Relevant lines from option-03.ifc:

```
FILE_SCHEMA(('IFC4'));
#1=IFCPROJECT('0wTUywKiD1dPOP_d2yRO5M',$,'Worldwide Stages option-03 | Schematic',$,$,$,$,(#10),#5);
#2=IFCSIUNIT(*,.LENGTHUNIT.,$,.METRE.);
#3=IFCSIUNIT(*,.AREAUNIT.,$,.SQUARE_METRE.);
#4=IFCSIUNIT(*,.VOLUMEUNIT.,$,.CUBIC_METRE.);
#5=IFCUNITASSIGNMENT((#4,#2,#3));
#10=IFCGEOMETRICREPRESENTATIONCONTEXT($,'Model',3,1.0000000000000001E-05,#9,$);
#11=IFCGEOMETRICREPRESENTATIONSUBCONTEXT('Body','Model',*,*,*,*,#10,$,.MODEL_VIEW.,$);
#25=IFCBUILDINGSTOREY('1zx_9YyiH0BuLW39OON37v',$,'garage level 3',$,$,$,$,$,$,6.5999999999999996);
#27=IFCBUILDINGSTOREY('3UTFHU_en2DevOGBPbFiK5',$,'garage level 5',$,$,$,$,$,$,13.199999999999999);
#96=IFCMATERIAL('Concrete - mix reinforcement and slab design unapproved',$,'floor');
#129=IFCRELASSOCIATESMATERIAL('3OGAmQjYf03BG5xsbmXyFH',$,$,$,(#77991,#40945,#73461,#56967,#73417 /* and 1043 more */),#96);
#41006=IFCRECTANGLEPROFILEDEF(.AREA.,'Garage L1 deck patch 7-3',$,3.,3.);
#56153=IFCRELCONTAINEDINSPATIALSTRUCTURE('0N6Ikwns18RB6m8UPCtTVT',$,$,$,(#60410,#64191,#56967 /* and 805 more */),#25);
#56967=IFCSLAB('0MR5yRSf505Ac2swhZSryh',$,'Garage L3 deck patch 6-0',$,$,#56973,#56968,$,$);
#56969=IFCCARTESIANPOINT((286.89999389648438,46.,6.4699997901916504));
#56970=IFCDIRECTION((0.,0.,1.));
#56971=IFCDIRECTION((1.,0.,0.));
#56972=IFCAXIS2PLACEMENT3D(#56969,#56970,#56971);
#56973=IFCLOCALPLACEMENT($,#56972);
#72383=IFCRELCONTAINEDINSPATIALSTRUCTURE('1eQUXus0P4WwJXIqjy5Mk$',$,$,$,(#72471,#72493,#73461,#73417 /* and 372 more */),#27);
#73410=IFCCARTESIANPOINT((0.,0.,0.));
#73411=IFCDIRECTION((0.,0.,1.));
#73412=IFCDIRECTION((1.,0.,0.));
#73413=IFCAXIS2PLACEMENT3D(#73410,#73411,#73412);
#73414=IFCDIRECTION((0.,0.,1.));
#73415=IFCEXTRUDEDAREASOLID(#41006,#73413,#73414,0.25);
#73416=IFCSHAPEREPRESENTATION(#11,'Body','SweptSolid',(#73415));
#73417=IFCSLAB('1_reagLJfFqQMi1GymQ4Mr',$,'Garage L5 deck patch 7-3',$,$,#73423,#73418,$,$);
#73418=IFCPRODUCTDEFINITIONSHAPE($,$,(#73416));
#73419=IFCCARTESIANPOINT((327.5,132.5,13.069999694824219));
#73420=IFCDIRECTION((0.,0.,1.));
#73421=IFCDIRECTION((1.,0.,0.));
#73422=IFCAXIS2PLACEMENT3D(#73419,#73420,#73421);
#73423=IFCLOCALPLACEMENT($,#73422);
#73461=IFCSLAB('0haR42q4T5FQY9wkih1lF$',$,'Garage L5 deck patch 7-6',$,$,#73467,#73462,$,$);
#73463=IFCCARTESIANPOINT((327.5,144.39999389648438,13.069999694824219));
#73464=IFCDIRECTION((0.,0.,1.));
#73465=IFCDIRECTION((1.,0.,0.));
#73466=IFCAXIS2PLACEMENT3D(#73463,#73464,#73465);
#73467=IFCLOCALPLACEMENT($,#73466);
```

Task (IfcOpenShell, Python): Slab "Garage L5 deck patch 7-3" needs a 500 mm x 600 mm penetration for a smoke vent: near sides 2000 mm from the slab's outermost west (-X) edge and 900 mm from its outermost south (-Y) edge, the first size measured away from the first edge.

```python
import numpy as np
import ifcopenshell
import ifcopenshell.api.feature
import ifcopenshell.api.geometry
import ifcopenshell.api.root
import ifcopenshell.geom
import ifcopenshell.util.placement
import ifcopenshell.util.representation
import ifcopenshell.util.shape
import ifcopenshell.util.unit

model = ifcopenshell.open("option-03.ifc")
unit_scale = ifcopenshell.util.unit.calculate_unit_scale(model)
settings = ifcopenshell.geom.settings()


def volume(element):
    """Net volume in cubic metres, openings subtracted."""
    shape = ifcopenshell.geom.create_shape(settings, element)
    return ifcopenshell.util.shape.get_volume(shape.geometry)


slab = model.by_guid("1_reagLJfFqQMi1GymQ4Mr")
before = volume(slab)

# Extent in the slab's own axes, in metres. The edges named are its -X and -Y sides.
slab_shape = ifcopenshell.geom.create_shape(settings, slab)
vertices = ifcopenshell.util.shape.get_vertices(slab_shape.geometry)
x_min, y_min, bottom = vertices.min(axis=0)
top = vertices[:, 2].max()

opening = ifcopenshell.api.root.create_entity(model, ifc_class="IfcOpeningElement", name="Smoke vent opening", predefined_type="OPENING")
context = ifcopenshell.util.representation.get_context(model, "Model", "Body", "MODEL_VIEW")
width, depth = 0.5, 0.6
outline = [(0.0, 0.0), (width, 0.0), (width, depth), (0.0, depth), (0.0, 0.0)]
# Overshoot both faces by 50 mm so the cut is clean.
shape = ifcopenshell.api.geometry.add_slab_representation(
    model, context=context, depth=top - bottom + 0.1, polyline=outline
)
ifcopenshell.api.geometry.assign_representation(model, product=opening, representation=shape)

matrix = ifcopenshell.util.placement.get_local_placement(slab.ObjectPlacement)
matrix[:, 3] = matrix @ np.append(np.array([x_min + 2, y_min + 0.9, bottom - 0.05]) / unit_scale, 1.0)
ifcopenshell.api.geometry.edit_object_placement(model, product=opening, matrix=matrix, is_si=False)
ifcopenshell.api.feature.add_feature(model, feature=opening, element=slab)

after = volume(slab)

print(f"slab volume {before:.3f} -> {after:.3f} m3")

model.write("option-03_edited.ifc")
```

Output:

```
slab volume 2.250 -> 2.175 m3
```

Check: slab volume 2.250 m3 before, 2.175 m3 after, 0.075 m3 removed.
